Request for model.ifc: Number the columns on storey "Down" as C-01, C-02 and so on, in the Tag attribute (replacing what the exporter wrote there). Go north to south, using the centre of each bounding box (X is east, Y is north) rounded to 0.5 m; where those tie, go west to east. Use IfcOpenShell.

First a look at what the model holds.

```python
import ifcopenshell
import ifcopenshell.util.element
import ifcopenshell.util.placement

model = ifcopenshell.open("model.ifc")
print(model.schema)
storey = next(s for s in model.by_type("IfcBuildingStorey") if s.Name == "Down")
columns = [e for e in ifcopenshell.util.element.get_decomposition(storey) if e.is_a("IfcColumn")]
for e in sorted(columns, key=lambda e: e.id()):
    origin = ifcopenshell.util.placement.get_local_placement(e.ObjectPlacement)[:3, 3]
    print(e.id(), e.Tag, e.Name, origin.round(2) + 0.0, sep=" | ")
```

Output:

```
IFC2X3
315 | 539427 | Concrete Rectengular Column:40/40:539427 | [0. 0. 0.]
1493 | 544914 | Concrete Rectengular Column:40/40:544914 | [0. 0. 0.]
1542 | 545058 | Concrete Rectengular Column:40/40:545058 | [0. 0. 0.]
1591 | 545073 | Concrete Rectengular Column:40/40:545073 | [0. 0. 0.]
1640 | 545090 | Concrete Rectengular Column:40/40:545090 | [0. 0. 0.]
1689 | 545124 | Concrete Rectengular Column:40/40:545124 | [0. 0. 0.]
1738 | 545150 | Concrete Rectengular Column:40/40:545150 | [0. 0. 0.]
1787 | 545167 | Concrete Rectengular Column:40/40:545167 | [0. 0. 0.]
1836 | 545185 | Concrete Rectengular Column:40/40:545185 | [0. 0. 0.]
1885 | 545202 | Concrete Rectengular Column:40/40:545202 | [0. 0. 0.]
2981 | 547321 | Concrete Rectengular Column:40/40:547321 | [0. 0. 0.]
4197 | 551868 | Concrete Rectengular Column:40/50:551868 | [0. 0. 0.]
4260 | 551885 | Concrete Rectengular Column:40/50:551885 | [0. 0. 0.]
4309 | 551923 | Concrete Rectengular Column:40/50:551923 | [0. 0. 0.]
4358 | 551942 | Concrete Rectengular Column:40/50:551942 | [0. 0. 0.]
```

```python
import ifcopenshell
import ifcopenshell.geom
import ifcopenshell.util.element
import ifcopenshell.util.shape

model = ifcopenshell.open("model.ifc")
settings = ifcopenshell.geom.settings()
settings.set("use-world-coords", True)


def centre(element):
    shape = ifcopenshell.geom.create_shape(settings, element)
    return ifcopenshell.util.shape.get_bbox_centroid(shape.geometry)


storey = next(s for s in model.by_type("IfcBuildingStorey") if s.Name == "Down")
columns = [e for e in ifcopenshell.util.element.get_decomposition(storey) if e.is_a("IfcColumn")]

# Insertion points can sit at a corner or the storey origin, so sort by the geometry (in metres).
centres = {e: centre(e) for e in columns}
columns.sort(key=lambda e: (-round(centres[e][1] / 0.5), centres[e][0]))

for i, e in enumerate(columns, start=1):
    number = f"C-{i:02d}"
    e.Tag = number
    print(e.id(), number)

model.write("model_updated.ifc")
```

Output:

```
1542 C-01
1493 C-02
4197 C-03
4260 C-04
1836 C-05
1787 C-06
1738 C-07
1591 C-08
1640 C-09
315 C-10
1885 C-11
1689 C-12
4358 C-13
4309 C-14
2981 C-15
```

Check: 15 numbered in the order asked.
